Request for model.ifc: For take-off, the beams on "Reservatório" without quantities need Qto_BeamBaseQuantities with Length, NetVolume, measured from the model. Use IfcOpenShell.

First a look at what the model holds.

```python
import ifcopenshell
import ifcopenshell.util.element
import ifcopenshell.util.unit

model = ifcopenshell.open("model.ifc")
print(model.schema)
for unit_type in ("LENGTHUNIT", "AREAUNIT", "VOLUMEUNIT"):
    print(unit_type, ifcopenshell.util.unit.calculate_unit_scale(model, unit_type))
storey = next(s for s in model.by_type("IfcBuildingStorey") if s.Name == "Reservatório")
beams = [e for e in ifcopenshell.util.element.get_decomposition(storey) if e.is_a("IfcBeam")]
for e in sorted(beams, key=lambda e: e.id()):
    print(e.id(), e.is_a(), e.Name, list(ifcopenshell.util.element.get_psets(e, qtos_only=True)), sep=" | ")
```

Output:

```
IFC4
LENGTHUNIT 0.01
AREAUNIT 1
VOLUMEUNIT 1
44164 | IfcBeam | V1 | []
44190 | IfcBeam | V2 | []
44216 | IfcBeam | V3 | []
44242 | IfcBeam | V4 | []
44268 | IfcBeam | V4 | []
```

```python
import ifcopenshell
import ifcopenshell.api.pset
import ifcopenshell.geom
import ifcopenshell.util.element
import ifcopenshell.util.shape
import ifcopenshell.util.unit

model = ifcopenshell.open("model.ifc")
unit_scale = ifcopenshell.util.unit.calculate_unit_scale(model)
volume_scale = ifcopenshell.util.unit.calculate_unit_scale(model, "VOLUMEUNIT")
settings = ifcopenshell.geom.settings()

storey = next(s for s in model.by_type("IfcBuildingStorey") if s.Name == "Reservatório")
beams = [e for e in ifcopenshell.util.element.get_decomposition(storey) if e.is_a("IfcBeam")]

for e in sorted(beams, key=lambda e: e.id()):
    if ifcopenshell.util.element.get_psets(e, qtos_only=True, should_inherit=False):
        continue
    # Geometry comes back in metres, in the element's own axes.
    shape = ifcopenshell.geom.create_shape(settings, e)
    values = {
        "Length": ifcopenshell.util.shape.get_max_xyz(shape.geometry) / unit_scale,
        "NetVolume": ifcopenshell.util.shape.get_volume(shape.geometry) / volume_scale,
    }
    qto = ifcopenshell.api.pset.add_qto(model, product=e, name="Qto_BeamBaseQuantities")
    ifcopenshell.api.pset.edit_qto(model, qto=qto, properties=values)
    print(e.id(), {k: round(v, 3) for k, v in values.items()})

model.write("model-out.ifc")
```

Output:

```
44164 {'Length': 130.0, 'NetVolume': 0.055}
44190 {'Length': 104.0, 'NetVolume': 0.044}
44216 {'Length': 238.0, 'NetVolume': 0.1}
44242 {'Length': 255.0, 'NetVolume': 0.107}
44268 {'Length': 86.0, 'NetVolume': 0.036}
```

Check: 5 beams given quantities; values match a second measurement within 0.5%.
